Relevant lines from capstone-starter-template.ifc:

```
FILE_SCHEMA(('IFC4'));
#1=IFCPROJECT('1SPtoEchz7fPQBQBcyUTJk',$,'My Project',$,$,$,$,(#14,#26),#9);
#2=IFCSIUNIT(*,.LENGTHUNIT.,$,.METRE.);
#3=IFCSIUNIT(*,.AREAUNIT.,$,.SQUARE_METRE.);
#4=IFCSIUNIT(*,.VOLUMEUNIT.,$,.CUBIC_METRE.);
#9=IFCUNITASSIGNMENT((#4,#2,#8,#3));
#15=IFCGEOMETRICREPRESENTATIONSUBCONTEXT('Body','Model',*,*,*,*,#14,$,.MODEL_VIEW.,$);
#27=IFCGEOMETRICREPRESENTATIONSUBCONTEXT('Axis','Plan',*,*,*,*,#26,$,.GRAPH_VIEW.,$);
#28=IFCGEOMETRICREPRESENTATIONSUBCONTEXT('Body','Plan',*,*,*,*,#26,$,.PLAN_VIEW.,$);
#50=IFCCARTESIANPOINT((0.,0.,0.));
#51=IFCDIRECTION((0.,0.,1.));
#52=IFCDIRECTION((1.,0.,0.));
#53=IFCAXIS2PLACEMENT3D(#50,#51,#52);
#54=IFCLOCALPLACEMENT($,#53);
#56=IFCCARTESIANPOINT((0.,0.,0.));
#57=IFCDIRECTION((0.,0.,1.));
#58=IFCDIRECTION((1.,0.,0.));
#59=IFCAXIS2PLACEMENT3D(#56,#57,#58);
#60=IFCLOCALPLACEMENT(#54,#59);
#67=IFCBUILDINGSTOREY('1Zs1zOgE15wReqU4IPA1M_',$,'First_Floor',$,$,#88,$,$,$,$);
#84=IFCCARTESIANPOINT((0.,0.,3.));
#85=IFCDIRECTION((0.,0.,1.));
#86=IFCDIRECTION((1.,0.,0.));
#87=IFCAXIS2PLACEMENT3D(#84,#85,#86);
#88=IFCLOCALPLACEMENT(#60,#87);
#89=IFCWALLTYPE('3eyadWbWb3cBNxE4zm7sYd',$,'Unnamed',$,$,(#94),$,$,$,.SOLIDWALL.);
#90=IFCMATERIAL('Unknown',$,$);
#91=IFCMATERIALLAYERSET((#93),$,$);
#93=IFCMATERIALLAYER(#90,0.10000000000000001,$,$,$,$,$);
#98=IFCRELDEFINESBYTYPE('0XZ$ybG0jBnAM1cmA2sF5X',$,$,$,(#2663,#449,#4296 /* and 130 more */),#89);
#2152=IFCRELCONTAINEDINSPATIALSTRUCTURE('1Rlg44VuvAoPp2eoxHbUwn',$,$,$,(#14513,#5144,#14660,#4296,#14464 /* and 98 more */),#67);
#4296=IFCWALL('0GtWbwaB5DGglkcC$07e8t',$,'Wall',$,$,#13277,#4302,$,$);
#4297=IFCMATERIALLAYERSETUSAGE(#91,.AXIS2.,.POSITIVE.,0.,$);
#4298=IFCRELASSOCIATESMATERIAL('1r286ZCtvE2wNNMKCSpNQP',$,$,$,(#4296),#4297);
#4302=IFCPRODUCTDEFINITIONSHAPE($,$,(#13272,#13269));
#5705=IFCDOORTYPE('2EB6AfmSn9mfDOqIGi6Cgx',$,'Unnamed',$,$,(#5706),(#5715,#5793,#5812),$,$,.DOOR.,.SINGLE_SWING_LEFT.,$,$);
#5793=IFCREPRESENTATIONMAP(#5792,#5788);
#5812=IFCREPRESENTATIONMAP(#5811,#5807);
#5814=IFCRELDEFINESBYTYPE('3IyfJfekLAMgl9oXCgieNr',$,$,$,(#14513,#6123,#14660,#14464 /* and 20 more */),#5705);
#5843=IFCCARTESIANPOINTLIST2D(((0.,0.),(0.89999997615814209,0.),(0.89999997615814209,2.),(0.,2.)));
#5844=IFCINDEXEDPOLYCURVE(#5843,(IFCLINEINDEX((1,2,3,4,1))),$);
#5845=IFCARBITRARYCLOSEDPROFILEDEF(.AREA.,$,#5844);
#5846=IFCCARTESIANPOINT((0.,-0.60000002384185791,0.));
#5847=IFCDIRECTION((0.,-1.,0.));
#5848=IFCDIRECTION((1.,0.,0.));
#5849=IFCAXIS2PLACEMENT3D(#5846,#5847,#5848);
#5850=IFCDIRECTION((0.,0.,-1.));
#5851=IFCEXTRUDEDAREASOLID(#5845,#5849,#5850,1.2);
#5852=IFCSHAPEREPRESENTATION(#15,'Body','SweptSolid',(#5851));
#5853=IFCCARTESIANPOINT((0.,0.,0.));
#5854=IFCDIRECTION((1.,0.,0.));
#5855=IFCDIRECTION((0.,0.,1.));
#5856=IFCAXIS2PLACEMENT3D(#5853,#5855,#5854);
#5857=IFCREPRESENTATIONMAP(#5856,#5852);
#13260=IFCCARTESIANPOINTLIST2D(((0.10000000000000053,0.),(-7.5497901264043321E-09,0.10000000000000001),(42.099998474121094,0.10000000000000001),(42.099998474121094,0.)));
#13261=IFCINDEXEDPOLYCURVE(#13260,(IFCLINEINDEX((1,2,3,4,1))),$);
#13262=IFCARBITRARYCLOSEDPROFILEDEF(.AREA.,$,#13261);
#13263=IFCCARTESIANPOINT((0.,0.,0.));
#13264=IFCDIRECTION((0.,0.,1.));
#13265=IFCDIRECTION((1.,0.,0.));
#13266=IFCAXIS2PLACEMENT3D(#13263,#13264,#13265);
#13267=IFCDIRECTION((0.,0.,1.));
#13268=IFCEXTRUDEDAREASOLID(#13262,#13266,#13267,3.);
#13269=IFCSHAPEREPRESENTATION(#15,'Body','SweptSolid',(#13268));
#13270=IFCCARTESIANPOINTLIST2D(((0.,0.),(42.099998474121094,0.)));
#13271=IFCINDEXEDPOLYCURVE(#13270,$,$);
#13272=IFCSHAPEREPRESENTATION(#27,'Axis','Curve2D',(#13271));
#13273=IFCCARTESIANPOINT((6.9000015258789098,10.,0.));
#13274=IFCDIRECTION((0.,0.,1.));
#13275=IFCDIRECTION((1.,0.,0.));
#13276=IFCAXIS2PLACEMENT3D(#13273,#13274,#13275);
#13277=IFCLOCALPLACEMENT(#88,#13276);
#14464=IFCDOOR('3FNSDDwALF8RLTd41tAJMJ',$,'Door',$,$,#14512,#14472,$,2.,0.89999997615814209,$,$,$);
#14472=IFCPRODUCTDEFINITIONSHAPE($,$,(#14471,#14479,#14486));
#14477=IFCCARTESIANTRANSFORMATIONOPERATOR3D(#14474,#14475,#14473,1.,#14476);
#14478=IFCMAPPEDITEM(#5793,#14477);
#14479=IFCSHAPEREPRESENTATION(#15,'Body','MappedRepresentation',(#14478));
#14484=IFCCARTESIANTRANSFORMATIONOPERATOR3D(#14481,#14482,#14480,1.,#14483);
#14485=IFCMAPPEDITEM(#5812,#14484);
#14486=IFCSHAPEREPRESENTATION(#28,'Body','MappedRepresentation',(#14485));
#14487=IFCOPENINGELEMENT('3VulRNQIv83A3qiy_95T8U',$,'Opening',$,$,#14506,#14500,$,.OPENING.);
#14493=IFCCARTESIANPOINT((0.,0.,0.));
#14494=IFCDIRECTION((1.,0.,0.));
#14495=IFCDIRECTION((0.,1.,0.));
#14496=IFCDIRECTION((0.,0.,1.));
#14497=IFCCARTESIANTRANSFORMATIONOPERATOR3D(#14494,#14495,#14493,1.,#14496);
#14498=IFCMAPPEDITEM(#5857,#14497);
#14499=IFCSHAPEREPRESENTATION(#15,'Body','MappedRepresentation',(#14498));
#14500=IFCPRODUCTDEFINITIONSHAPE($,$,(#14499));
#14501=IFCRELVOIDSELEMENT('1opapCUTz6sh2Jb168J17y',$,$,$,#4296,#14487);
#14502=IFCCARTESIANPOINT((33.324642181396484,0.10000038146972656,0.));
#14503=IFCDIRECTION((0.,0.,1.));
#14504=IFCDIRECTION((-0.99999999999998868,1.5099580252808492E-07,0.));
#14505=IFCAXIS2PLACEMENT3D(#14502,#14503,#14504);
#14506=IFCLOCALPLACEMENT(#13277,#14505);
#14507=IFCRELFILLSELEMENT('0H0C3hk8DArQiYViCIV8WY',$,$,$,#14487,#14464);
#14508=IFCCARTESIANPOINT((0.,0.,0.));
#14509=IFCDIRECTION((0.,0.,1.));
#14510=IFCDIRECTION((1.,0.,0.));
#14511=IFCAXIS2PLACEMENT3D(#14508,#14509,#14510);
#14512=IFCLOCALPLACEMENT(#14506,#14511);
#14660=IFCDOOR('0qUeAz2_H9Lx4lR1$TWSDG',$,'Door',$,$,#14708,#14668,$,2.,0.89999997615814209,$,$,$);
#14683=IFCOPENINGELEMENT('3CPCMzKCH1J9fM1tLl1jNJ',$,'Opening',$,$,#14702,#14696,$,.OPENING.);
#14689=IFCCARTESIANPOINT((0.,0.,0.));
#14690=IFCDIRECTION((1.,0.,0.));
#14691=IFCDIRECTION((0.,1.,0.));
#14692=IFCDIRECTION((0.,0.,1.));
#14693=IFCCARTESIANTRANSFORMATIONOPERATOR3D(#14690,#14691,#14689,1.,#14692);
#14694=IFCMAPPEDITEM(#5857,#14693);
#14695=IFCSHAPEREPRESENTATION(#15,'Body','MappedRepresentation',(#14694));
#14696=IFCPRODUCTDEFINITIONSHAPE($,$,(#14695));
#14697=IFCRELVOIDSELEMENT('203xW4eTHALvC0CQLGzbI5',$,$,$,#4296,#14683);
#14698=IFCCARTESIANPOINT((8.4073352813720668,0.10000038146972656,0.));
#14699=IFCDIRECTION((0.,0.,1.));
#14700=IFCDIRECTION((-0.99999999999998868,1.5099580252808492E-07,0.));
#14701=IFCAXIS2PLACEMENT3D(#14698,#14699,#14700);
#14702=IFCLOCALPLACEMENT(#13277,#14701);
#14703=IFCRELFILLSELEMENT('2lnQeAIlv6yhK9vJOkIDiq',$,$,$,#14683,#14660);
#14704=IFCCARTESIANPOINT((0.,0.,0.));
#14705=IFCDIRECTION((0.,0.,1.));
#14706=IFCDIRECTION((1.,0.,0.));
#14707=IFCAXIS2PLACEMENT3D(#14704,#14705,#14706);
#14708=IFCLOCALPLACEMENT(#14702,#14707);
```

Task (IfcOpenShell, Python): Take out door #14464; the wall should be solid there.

```python
import ifcopenshell
import ifcopenshell.api.feature
import ifcopenshell.api.root
import ifcopenshell.geom
import ifcopenshell.util.shape

model = ifcopenshell.open("capstone-starter-template.ifc")
settings = ifcopenshell.geom.settings()


def volume(element):
    """Net volume in cubic metres, openings subtracted."""
    shape = ifcopenshell.geom.create_shape(settings, element)
    return ifcopenshell.util.shape.get_volume(shape.geometry)


door = model.by_id(14464)
opening = door.FillsVoids[0].RelatingOpeningElement
wall = opening.VoidsElements[0].RelatingBuildingElement
before = volume(wall)

ifcopenshell.api.root.remove_product(model, product=door)
ifcopenshell.api.feature.remove_feature(model, feature=opening)

after = volume(wall)

print(f"wall volume {before:.3f} -> {after:.3f} m3")

model.write("capstone-starter-template_rev.ifc")
```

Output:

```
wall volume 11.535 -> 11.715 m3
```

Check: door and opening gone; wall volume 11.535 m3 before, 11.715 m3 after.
